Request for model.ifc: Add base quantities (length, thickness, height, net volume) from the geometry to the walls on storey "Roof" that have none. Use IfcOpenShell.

First a look at what the model holds.

```python
import ifcopenshell
import ifcopenshell.util.element
import ifcopenshell.util.unit

model = ifcopenshell.open("model.ifc")
print(model.schema)
for unit_type in ("LENGTHUNIT", "AREAUNIT", "VOLUMEUNIT"):
    print(unit_type, ifcopenshell.util.unit.calculate_unit_scale(model, unit_type))
storey = next(s for s in model.by_type("IfcBuildingStorey") if s.Name == "Roof")
walls = [e for e in ifcopenshell.util.element.get_decomposition(storey) if e.is_a("IfcWall")]
for e in sorted(walls, key=lambda e: e.id()):
    print(e.id(), e.is_a(), e.Name, list(ifcopenshell.util.element.get_psets(e, qtos_only=True)), sep=" | ")
```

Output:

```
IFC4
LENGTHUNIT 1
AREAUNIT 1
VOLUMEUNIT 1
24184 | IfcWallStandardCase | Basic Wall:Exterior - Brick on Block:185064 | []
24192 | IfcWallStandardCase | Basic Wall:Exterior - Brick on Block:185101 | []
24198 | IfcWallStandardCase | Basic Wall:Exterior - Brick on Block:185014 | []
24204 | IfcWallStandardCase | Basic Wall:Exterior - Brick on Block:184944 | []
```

```python
import ifcopenshell
import ifcopenshell.api.pset
import ifcopenshell.geom
import ifcopenshell.util.element
import ifcopenshell.util.shape
import ifcopenshell.util.unit

model = ifcopenshell.open("model.ifc")
unit_scale = ifcopenshell.util.unit.calculate_unit_scale(model)
volume_scale = ifcopenshell.util.unit.calculate_unit_scale(model, "VOLUMEUNIT")
settings = ifcopenshell.geom.settings()

storey = next(s for s in model.by_type("IfcBuildingStorey") if s.Name == "Roof")
walls = [e for e in ifcopenshell.util.element.get_decomposition(storey) if e.is_a("IfcWall")]

for e in sorted(walls, key=lambda e: e.id()):
    if ifcopenshell.util.element.get_psets(e, qtos_only=True, should_inherit=False):
        continue
    # Geometry comes back in metres, in the element's own axes.
    shape = ifcopenshell.geom.create_shape(settings, e)
    values = {
        "Length": ifcopenshell.util.shape.get_x(shape.geometry) / unit_scale,
        "Width": ifcopenshell.util.shape.get_y(shape.geometry) / unit_scale,
        "Height": ifcopenshell.util.shape.get_z(shape.geometry) / unit_scale,
        "NetVolume": ifcopenshell.util.shape.get_volume(shape.geometry) / volume_scale,
    }
    qto = ifcopenshell.api.pset.add_qto(model, product=e, name="Qto_WallBaseQuantities")
    ifcopenshell.api.pset.edit_qto(model, qto=qto, properties=values)
    print(e.id(), {k: round(v, 3) for k, v in values.items()})

model.write("model_edited.ifc")
```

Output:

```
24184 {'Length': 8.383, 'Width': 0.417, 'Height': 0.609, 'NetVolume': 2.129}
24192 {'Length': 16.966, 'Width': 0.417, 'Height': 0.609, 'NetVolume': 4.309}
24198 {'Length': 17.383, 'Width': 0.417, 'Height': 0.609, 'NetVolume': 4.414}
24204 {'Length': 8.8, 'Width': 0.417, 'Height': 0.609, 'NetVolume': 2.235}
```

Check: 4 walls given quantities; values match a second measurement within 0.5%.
